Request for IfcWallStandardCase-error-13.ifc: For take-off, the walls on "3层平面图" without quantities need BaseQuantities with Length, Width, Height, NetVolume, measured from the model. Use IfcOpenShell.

First a look at what the model holds.

```python
import ifcopenshell
import ifcopenshell.util.element
import ifcopenshell.util.unit

model = ifcopenshell.open("IfcWallStandardCase-error-13.ifc")
print(model.schema)
for unit_type in ("LENGTHUNIT", "AREAUNIT", "VOLUMEUNIT"):
    print(unit_type, ifcopenshell.util.unit.calculate_unit_scale(model, unit_type))
storey = next(s for s in model.by_type("IfcBuildingStorey") if s.Name == "3层平面图")
walls = [e for e in ifcopenshell.util.element.get_decomposition(storey) if e.is_a("IfcWall")]
for e in sorted(walls, key=lambda e: e.id()):
    print(e.id(), e.is_a(), e.Name, list(ifcopenshell.util.element.get_psets(e, qtos_only=True)), sep=" | ")
```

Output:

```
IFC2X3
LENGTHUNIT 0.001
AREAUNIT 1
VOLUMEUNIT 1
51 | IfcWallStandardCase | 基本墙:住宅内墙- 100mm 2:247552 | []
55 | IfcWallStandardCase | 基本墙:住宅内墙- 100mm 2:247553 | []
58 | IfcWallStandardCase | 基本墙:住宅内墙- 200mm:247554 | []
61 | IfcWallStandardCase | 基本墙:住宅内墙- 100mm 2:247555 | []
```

```python
import ifcopenshell
import ifcopenshell.api.pset
import ifcopenshell.geom
import ifcopenshell.util.element
import ifcopenshell.util.shape
import ifcopenshell.util.unit

model = ifcopenshell.open("IfcWallStandardCase-error-13.ifc")
unit_scale = ifcopenshell.util.unit.calculate_unit_scale(model)
volume_scale = ifcopenshell.util.unit.calculate_unit_scale(model, "VOLUMEUNIT")
settings = ifcopenshell.geom.settings()

storey = next(s for s in model.by_type("IfcBuildingStorey") if s.Name == "3层平面图")
walls = [e for e in ifcopenshell.util.element.get_decomposition(storey) if e.is_a("IfcWall")]

for e in sorted(walls, key=lambda e: e.id()):
    if ifcopenshell.util.element.get_psets(e, qtos_only=True, should_inherit=False):
        continue
    # Geometry comes back in metres, in the element's own axes.
    shape = ifcopenshell.geom.create_shape(settings, e)
    values = {
        "Length": ifcopenshell.util.shape.get_x(shape.geometry) / unit_scale,
        "Width": ifcopenshell.util.shape.get_y(shape.geometry) / unit_scale,
        "Height": ifcopenshell.util.shape.get_z(shape.geometry) / unit_scale,
        "NetVolume": ifcopenshell.util.shape.get_volume(shape.geometry) / volume_scale,
    }
    qto = ifcopenshell.api.pset.add_qto(model, product=e, name="BaseQuantities")
    ifcopenshell.api.pset.edit_qto(model, qto=qto, properties=values)
    print(e.id(), {k: round(v, 3) for k, v in values.items()})

model.write("IfcWallStandardCase-error-13_updated.ifc")
```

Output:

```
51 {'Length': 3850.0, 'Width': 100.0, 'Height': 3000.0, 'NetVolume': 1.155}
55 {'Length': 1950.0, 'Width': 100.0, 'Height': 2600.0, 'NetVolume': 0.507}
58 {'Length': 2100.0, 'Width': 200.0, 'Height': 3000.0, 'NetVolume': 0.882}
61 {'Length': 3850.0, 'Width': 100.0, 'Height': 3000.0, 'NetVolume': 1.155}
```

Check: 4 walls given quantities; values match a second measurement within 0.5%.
